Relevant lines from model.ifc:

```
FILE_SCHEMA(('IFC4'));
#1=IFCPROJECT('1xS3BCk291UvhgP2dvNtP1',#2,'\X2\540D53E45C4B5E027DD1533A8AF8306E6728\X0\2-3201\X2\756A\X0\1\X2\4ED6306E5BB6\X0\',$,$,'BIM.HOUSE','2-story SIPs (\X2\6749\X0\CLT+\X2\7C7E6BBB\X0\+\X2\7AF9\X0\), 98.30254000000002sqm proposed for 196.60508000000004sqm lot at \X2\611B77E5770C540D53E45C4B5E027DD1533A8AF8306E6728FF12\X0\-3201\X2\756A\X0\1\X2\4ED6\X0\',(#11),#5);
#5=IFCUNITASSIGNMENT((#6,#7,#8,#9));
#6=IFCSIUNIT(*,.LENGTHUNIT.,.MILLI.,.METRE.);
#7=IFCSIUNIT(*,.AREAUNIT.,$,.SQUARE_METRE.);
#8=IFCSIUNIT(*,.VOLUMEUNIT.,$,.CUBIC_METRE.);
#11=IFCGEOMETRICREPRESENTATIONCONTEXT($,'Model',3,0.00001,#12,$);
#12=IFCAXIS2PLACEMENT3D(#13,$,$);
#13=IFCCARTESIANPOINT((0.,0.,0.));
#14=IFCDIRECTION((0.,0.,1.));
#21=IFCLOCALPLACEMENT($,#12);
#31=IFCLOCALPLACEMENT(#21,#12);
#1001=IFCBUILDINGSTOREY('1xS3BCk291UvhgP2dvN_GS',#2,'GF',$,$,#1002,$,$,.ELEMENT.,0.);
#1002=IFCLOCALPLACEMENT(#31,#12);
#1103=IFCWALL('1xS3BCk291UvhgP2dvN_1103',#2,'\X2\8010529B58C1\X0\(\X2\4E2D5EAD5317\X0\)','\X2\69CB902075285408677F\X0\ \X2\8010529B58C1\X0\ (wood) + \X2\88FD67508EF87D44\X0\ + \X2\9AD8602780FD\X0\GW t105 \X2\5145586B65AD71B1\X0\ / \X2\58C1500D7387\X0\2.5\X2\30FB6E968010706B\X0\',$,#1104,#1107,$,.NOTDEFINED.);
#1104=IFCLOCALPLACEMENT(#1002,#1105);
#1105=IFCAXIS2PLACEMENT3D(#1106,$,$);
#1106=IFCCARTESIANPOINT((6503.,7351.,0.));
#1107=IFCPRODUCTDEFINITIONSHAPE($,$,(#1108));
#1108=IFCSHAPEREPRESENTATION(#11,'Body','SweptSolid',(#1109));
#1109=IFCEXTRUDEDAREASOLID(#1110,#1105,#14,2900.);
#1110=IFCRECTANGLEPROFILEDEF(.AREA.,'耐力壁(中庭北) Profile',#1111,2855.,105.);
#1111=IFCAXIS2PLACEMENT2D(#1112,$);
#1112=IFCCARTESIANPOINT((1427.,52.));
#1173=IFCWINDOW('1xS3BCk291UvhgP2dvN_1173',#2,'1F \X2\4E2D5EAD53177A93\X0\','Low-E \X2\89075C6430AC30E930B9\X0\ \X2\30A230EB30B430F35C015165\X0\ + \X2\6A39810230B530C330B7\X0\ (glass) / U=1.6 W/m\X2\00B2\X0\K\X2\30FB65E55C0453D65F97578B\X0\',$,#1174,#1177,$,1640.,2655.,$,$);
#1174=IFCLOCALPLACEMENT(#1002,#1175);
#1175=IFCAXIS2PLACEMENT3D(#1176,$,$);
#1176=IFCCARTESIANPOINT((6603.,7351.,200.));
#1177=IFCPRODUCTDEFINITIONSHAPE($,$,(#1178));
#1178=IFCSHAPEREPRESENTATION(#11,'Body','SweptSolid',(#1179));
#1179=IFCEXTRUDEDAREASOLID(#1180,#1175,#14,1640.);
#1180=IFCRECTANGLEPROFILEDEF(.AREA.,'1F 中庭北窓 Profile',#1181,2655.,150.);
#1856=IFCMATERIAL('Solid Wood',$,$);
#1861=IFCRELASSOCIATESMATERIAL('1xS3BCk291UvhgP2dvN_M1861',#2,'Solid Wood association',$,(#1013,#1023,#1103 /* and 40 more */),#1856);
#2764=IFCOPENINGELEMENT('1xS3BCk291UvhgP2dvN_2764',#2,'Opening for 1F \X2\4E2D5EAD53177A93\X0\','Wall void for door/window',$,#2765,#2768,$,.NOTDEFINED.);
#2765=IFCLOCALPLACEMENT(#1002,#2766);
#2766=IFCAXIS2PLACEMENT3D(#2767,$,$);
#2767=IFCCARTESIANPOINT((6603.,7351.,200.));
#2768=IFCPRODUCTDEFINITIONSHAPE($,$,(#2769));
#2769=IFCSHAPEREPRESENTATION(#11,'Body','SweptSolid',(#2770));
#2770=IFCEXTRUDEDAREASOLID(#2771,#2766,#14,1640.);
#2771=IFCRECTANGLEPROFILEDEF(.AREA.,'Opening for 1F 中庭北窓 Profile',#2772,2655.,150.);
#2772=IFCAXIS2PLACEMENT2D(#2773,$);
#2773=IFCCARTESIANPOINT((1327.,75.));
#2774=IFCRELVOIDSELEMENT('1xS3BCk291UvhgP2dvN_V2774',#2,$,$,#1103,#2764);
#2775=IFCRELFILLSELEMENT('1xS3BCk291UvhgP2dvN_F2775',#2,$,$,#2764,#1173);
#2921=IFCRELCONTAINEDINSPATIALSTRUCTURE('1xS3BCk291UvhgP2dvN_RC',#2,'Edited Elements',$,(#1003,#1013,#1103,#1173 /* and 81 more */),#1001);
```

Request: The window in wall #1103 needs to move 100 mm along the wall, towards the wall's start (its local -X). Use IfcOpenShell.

```python
import ifcopenshell
import ifcopenshell.api.geometry
import ifcopenshell.util.placement
import ifcopenshell.util.unit

model = ifcopenshell.open("model.ifc")
unit_scale = ifcopenshell.util.unit.calculate_unit_scale(model)

window = model.by_guid("1xS3BCk291UvhgP2dvN_1173")
opening = window.FillsVoids[0].RelatingOpeningElement
wall = opening.VoidsElements[0].RelatingBuildingElement

wall_matrix = ifcopenshell.util.placement.get_local_placement(wall.ObjectPlacement)
shift = wall_matrix[:3, 0] * -0.1 / unit_scale
before = ifcopenshell.util.placement.get_local_placement(window.ObjectPlacement)[:3, 3].copy()

# The window is not placed relative to its opening, so move both.
for product in (opening, window):
    matrix = ifcopenshell.util.placement.get_local_placement(product.ObjectPlacement)
    matrix[:3, 3] += shift
    ifcopenshell.api.geometry.edit_object_placement(model, product=product, matrix=matrix, is_si=False)

after = ifcopenshell.util.placement.get_local_placement(window.ObjectPlacement)[:3, 3]
print("window moved by", (after - before).round(3) + 0.0)

model.write("model_updated.ifc")
```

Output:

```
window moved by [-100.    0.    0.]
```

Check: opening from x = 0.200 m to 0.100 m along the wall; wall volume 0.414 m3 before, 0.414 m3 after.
